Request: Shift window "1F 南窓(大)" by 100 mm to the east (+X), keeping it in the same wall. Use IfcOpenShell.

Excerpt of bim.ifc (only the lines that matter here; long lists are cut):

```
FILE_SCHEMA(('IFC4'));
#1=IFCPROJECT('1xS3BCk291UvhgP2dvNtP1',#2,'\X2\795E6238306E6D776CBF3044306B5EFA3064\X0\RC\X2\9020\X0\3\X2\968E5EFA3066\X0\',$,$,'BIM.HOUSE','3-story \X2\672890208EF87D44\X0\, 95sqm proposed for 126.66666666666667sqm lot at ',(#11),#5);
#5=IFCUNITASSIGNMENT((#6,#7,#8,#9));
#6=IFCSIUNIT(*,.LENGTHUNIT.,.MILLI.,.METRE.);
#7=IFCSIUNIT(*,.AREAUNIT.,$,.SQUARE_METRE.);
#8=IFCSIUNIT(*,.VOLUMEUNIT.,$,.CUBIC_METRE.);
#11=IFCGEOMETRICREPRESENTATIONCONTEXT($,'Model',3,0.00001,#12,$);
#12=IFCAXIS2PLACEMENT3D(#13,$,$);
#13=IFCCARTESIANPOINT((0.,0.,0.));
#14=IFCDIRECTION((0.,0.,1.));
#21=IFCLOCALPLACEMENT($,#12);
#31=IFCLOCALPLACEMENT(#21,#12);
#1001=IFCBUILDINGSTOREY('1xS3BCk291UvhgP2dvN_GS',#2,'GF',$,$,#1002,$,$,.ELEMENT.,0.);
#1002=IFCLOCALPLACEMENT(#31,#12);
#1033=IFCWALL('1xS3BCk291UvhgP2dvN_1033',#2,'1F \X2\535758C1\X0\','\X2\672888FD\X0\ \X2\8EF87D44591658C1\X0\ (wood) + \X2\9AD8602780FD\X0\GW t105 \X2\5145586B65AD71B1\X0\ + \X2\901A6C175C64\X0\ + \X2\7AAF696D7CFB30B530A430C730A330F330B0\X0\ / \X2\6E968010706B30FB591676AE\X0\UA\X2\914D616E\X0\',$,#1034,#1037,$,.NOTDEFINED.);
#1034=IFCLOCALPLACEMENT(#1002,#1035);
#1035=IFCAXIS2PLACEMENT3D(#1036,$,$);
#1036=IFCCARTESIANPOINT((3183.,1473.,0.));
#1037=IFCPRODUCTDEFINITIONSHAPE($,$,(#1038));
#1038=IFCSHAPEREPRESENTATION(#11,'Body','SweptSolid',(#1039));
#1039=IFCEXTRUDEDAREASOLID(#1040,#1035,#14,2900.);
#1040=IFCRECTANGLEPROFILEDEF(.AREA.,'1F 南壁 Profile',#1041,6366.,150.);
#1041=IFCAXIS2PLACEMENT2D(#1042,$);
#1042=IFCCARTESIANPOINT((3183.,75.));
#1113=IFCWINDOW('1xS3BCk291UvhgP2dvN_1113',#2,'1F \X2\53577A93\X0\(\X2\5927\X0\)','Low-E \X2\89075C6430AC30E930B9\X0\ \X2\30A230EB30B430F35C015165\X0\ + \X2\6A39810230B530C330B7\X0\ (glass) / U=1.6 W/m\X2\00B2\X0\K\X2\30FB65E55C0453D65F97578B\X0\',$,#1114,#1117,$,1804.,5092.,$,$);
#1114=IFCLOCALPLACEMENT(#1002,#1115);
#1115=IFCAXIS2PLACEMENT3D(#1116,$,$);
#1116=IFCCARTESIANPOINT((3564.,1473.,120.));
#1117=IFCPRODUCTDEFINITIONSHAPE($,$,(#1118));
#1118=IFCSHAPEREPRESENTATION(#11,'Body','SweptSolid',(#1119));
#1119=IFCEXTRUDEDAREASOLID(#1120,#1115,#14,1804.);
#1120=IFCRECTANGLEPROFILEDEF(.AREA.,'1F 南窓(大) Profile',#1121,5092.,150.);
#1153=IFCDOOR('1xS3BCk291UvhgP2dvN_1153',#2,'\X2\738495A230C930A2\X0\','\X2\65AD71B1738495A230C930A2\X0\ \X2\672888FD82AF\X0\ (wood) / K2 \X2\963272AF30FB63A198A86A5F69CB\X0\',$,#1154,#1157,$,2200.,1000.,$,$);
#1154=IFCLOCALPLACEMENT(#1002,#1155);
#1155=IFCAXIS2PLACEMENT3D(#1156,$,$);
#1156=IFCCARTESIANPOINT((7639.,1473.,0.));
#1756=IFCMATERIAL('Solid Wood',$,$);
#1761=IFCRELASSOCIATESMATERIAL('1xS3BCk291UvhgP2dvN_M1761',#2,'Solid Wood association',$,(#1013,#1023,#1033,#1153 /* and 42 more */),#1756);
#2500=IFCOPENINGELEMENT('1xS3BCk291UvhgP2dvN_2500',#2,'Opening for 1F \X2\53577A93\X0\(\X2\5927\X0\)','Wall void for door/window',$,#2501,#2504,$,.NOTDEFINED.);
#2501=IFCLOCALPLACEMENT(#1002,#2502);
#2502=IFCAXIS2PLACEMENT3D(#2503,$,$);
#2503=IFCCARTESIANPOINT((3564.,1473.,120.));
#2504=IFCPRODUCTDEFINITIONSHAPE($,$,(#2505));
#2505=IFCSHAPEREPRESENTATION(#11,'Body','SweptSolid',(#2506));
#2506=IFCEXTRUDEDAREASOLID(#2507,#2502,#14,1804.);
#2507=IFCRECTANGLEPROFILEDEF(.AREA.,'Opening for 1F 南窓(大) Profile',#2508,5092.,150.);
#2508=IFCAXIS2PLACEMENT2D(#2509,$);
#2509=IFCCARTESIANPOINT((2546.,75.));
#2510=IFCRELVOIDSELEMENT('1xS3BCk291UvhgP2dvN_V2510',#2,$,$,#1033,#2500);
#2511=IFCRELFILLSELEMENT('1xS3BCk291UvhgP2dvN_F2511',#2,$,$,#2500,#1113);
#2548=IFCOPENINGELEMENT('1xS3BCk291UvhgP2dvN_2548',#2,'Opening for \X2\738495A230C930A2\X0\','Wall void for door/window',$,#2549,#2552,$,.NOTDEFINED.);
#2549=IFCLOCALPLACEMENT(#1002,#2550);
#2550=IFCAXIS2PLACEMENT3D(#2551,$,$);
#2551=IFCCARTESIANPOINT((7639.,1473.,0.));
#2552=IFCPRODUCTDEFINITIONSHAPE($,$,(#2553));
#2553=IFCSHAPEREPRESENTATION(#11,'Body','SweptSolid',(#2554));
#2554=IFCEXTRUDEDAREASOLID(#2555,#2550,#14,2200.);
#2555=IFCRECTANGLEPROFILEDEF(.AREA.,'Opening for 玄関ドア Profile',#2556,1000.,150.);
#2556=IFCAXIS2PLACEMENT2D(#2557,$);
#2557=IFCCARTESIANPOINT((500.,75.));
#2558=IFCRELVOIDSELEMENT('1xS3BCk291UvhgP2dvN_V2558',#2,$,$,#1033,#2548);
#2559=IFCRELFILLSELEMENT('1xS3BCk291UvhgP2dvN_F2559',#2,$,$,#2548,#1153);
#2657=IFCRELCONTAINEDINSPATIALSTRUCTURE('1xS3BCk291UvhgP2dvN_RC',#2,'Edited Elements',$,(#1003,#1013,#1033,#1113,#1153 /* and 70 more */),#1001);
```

```python
import ifcopenshell
import ifcopenshell.api.geometry
import ifcopenshell.util.placement

model = ifcopenshell.open("bim.ifc")

window = model.by_guid("1xS3BCk291UvhgP2dvN_1113")
opening = window.FillsVoids[0].RelatingOpeningElement
wall = opening.VoidsElements[0].RelatingBuildingElement

wall_matrix = ifcopenshell.util.placement.get_local_placement(wall.ObjectPlacement)
shift = wall_matrix[:3, 0] * 100.0
before = ifcopenshell.util.placement.get_local_placement(window.ObjectPlacement)[:3, 3].copy()

# The window is not placed relative to its opening, so move both.
for product in (opening, window):
    matrix = ifcopenshell.util.placement.get_local_placement(product.ObjectPlacement)
    matrix[:3, 3] += shift
    ifcopenshell.api.geometry.edit_object_placement(model, product=product, matrix=matrix, is_si=False)

after = ifcopenshell.util.placement.get_local_placement(window.ObjectPlacement)[:3, 3]
print("window moved by", (after - before).round(3) + 0.0)

model.write("bim-out.ifc")
```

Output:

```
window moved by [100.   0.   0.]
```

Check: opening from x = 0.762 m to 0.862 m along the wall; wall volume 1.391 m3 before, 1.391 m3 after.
